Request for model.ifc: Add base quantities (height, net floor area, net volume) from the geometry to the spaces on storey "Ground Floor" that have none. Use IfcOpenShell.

First a look at what the model holds.

```python
import ifcopenshell
import ifcopenshell.util.element
import ifcopenshell.util.unit

model = ifcopenshell.open("model.ifc")
print(model.schema)
for unit_type in ("LENGTHUNIT", "AREAUNIT", "VOLUMEUNIT"):
    print(unit_type, ifcopenshell.util.unit.calculate_unit_scale(model, unit_type))
storey = next(s for s in model.by_type("IfcBuildingStorey") if s.Name == "Ground Floor")
spaces = [e for e in ifcopenshell.util.element.get_decomposition(storey) if e.is_a("IfcSpace")]
for e in sorted(spaces, key=lambda e: e.id()):
    print(e.id(), e.is_a(), e.Name, list(ifcopenshell.util.element.get_psets(e, qtos_only=True)), sep=" | ")
```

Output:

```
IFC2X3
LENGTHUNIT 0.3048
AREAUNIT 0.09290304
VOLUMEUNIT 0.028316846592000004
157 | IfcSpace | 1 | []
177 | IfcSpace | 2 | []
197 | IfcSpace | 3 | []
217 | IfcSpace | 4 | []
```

```python
import ifcopenshell
import ifcopenshell.api.pset
import ifcopenshell.geom
import ifcopenshell.util.element
import ifcopenshell.util.shape
import ifcopenshell.util.unit

model = ifcopenshell.open("model.ifc")
unit_scale = ifcopenshell.util.unit.calculate_unit_scale(model)
area_scale = ifcopenshell.util.unit.calculate_unit_scale(model, "AREAUNIT")
volume_scale = ifcopenshell.util.unit.calculate_unit_scale(model, "VOLUMEUNIT")
settings = ifcopenshell.geom.settings()

storey = next(s for s in model.by_type("IfcBuildingStorey") if s.Name == "Ground Floor")
spaces = [e for e in ifcopenshell.util.element.get_decomposition(storey) if e.is_a("IfcSpace")]

for e in sorted(spaces, key=lambda e: e.id()):
    if ifcopenshell.util.element.get_psets(e, qtos_only=True, should_inherit=False):
        continue
    # Geometry comes back in metres, in the element's own axes.
    shape = ifcopenshell.geom.create_shape(settings, e)
    values = {
        "Height": ifcopenshell.util.shape.get_z(shape.geometry) / unit_scale,
        "NetFloorArea": ifcopenshell.util.shape.get_footprint_area(shape.geometry) / area_scale,
        "NetVolume": ifcopenshell.util.shape.get_volume(shape.geometry) / volume_scale,
    }
    qto = ifcopenshell.api.pset.add_qto(model, product=e, name="BaseQuantities")
    ifcopenshell.api.pset.edit_qto(model, qto=qto, properties=values)
    print(e.id(), {k: round(v, 3) for k, v in values.items()})

model.write("model_rev.ifc")
```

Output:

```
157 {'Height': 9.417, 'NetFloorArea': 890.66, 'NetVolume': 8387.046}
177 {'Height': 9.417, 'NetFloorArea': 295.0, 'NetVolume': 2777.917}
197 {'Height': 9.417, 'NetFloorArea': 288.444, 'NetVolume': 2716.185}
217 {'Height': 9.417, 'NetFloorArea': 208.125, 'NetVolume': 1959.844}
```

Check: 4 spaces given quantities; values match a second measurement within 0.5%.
